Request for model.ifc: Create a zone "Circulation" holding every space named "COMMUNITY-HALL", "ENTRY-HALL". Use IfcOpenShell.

First a look at what the model holds.

```python
import ifcopenshell

model = ifcopenshell.open("model.ifc")
print(model.schema)
seen = {}
for space in model.by_type("IfcSpace"):
    seen[space.Name] = seen.get(space.Name, 0) + 1
for name, count in sorted(seen.items(), key=str):
    print(count, "x", name)
print("zones:", [z.Name for z in model.by_type("IfcZone")][:20])
```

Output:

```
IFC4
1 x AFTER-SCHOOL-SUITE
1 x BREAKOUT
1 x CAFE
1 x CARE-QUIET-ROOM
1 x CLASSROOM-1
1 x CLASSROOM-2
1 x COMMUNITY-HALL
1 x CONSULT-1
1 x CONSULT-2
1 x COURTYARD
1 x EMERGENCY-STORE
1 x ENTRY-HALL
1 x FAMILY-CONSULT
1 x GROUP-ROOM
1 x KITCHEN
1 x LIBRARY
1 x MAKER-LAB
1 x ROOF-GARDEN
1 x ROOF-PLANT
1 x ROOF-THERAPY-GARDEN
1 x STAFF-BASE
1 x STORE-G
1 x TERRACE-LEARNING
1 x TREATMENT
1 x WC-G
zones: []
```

```python
import ifcopenshell
import ifcopenshell.api.group
import ifcopenshell.api.root

model = ifcopenshell.open("model.ifc")

names = {"COMMUNITY-HALL", "ENTRY-HALL"}
spaces = [s for s in model.by_type("IfcSpace") if s.Name in names]

zone = ifcopenshell.api.root.create_entity(model, ifc_class="IfcZone", name="Circulation")
ifcopenshell.api.group.assign_group(model, products=spaces, group=zone)
print(len(spaces), "spaces in", zone.Name)

model.write("model_v2.ifc")
```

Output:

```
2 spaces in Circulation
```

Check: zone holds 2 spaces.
